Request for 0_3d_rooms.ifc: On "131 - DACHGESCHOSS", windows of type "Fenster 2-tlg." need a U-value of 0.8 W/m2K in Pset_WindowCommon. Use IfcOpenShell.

First a look at what the model holds.

```python
import ifcopenshell
import ifcopenshell.util.element

model = ifcopenshell.open("0_3d_rooms.ifc")
print(model.schema)
storey = next(s for s in model.by_type("IfcBuildingStorey") if s.Name == "131 - DACHGESCHOSS")
windows = [e for e in ifcopenshell.util.element.get_decomposition(storey) if e.is_a("IfcWindow")]
seen = {}
for e in windows:
    element_type = ifcopenshell.util.element.get_type(e)
    key = (element_type.Name if element_type != e and element_type else None, ifcopenshell.util.element.get_pset(e, "Pset_WindowCommon", "ThermalTransmittance"))
    seen[key] = seen.get(key, 0) + 1
for (name, value), count in sorted(seen.items(), key=str):
    print(count, "x", name, "|", value)
```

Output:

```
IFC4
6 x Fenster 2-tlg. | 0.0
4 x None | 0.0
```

```python
import ifcopenshell
import ifcopenshell.api.pset
import ifcopenshell.util.element

model = ifcopenshell.open("0_3d_rooms.ifc")

storey = next(s for s in model.by_type("IfcBuildingStorey") if s.Name == "131 - DACHGESCHOSS")
windows = [e for e in ifcopenshell.util.element.get_decomposition(storey) if e.is_a("IfcWindow")]

count = 0
for e in windows:
    element_type = ifcopenshell.util.element.get_type(e)
    if element_type in (None, e) or element_type.Name != "Fenster 2-tlg.":
        continue
    # add_pset returns the element's existing set when there is one.
    pset = ifcopenshell.api.pset.add_pset(model, product=e, name="Pset_WindowCommon")
    ifcopenshell.api.pset.edit_pset(model, pset=pset, properties={"ThermalTransmittance": 0.8})
    count += 1

print(count, "windows updated")

model.write("0_3d_rooms_v2.ifc")
```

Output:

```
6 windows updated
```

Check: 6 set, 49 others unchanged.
